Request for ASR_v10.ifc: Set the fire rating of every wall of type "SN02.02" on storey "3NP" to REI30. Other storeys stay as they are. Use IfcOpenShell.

First a look at what the model holds.

```python
import ifcopenshell
import ifcopenshell.util.element

model = ifcopenshell.open("ASR_v10.ifc")
print(model.schema)
storey = next(s for s in model.by_type("IfcBuildingStorey") if s.Name == "3NP")
walls = [e for e in ifcopenshell.util.element.get_decomposition(storey) if e.is_a("IfcWall")]
seen = {}
for e in walls:
    element_type = ifcopenshell.util.element.get_type(e)
    key = (element_type.Name if element_type != e and element_type else None, ifcopenshell.util.element.get_pset(e, "Pset_WallCommon", "FireRating"))
    seen[key] = seen.get(key, 0) + 1
for (name, value), count in sorted(seen.items(), key=str):
    print(count, "x", name, "|", value)
```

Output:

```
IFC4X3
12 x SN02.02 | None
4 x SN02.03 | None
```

```python
import ifcopenshell
import ifcopenshell.api.pset
import ifcopenshell.util.element

model = ifcopenshell.open("ASR_v10.ifc")

storey = next(s for s in model.by_type("IfcBuildingStorey") if s.Name == "3NP")
walls = [e for e in ifcopenshell.util.element.get_decomposition(storey) if e.is_a("IfcWall")]

count = 0
for e in walls:
    element_type = ifcopenshell.util.element.get_type(e)
    if element_type in (None, e) or element_type.Name != "SN02.02":
        continue
    # add_pset returns the element's existing set when there is one.
    pset = ifcopenshell.api.pset.add_pset(model, product=e, name="Pset_WallCommon")
    ifcopenshell.api.pset.edit_pset(model, pset=pset, properties={"FireRating": "REI30"})
    count += 1

print(count, "walls updated")

model.write("ASR_v10_v2.ifc")
```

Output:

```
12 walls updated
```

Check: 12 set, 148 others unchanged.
